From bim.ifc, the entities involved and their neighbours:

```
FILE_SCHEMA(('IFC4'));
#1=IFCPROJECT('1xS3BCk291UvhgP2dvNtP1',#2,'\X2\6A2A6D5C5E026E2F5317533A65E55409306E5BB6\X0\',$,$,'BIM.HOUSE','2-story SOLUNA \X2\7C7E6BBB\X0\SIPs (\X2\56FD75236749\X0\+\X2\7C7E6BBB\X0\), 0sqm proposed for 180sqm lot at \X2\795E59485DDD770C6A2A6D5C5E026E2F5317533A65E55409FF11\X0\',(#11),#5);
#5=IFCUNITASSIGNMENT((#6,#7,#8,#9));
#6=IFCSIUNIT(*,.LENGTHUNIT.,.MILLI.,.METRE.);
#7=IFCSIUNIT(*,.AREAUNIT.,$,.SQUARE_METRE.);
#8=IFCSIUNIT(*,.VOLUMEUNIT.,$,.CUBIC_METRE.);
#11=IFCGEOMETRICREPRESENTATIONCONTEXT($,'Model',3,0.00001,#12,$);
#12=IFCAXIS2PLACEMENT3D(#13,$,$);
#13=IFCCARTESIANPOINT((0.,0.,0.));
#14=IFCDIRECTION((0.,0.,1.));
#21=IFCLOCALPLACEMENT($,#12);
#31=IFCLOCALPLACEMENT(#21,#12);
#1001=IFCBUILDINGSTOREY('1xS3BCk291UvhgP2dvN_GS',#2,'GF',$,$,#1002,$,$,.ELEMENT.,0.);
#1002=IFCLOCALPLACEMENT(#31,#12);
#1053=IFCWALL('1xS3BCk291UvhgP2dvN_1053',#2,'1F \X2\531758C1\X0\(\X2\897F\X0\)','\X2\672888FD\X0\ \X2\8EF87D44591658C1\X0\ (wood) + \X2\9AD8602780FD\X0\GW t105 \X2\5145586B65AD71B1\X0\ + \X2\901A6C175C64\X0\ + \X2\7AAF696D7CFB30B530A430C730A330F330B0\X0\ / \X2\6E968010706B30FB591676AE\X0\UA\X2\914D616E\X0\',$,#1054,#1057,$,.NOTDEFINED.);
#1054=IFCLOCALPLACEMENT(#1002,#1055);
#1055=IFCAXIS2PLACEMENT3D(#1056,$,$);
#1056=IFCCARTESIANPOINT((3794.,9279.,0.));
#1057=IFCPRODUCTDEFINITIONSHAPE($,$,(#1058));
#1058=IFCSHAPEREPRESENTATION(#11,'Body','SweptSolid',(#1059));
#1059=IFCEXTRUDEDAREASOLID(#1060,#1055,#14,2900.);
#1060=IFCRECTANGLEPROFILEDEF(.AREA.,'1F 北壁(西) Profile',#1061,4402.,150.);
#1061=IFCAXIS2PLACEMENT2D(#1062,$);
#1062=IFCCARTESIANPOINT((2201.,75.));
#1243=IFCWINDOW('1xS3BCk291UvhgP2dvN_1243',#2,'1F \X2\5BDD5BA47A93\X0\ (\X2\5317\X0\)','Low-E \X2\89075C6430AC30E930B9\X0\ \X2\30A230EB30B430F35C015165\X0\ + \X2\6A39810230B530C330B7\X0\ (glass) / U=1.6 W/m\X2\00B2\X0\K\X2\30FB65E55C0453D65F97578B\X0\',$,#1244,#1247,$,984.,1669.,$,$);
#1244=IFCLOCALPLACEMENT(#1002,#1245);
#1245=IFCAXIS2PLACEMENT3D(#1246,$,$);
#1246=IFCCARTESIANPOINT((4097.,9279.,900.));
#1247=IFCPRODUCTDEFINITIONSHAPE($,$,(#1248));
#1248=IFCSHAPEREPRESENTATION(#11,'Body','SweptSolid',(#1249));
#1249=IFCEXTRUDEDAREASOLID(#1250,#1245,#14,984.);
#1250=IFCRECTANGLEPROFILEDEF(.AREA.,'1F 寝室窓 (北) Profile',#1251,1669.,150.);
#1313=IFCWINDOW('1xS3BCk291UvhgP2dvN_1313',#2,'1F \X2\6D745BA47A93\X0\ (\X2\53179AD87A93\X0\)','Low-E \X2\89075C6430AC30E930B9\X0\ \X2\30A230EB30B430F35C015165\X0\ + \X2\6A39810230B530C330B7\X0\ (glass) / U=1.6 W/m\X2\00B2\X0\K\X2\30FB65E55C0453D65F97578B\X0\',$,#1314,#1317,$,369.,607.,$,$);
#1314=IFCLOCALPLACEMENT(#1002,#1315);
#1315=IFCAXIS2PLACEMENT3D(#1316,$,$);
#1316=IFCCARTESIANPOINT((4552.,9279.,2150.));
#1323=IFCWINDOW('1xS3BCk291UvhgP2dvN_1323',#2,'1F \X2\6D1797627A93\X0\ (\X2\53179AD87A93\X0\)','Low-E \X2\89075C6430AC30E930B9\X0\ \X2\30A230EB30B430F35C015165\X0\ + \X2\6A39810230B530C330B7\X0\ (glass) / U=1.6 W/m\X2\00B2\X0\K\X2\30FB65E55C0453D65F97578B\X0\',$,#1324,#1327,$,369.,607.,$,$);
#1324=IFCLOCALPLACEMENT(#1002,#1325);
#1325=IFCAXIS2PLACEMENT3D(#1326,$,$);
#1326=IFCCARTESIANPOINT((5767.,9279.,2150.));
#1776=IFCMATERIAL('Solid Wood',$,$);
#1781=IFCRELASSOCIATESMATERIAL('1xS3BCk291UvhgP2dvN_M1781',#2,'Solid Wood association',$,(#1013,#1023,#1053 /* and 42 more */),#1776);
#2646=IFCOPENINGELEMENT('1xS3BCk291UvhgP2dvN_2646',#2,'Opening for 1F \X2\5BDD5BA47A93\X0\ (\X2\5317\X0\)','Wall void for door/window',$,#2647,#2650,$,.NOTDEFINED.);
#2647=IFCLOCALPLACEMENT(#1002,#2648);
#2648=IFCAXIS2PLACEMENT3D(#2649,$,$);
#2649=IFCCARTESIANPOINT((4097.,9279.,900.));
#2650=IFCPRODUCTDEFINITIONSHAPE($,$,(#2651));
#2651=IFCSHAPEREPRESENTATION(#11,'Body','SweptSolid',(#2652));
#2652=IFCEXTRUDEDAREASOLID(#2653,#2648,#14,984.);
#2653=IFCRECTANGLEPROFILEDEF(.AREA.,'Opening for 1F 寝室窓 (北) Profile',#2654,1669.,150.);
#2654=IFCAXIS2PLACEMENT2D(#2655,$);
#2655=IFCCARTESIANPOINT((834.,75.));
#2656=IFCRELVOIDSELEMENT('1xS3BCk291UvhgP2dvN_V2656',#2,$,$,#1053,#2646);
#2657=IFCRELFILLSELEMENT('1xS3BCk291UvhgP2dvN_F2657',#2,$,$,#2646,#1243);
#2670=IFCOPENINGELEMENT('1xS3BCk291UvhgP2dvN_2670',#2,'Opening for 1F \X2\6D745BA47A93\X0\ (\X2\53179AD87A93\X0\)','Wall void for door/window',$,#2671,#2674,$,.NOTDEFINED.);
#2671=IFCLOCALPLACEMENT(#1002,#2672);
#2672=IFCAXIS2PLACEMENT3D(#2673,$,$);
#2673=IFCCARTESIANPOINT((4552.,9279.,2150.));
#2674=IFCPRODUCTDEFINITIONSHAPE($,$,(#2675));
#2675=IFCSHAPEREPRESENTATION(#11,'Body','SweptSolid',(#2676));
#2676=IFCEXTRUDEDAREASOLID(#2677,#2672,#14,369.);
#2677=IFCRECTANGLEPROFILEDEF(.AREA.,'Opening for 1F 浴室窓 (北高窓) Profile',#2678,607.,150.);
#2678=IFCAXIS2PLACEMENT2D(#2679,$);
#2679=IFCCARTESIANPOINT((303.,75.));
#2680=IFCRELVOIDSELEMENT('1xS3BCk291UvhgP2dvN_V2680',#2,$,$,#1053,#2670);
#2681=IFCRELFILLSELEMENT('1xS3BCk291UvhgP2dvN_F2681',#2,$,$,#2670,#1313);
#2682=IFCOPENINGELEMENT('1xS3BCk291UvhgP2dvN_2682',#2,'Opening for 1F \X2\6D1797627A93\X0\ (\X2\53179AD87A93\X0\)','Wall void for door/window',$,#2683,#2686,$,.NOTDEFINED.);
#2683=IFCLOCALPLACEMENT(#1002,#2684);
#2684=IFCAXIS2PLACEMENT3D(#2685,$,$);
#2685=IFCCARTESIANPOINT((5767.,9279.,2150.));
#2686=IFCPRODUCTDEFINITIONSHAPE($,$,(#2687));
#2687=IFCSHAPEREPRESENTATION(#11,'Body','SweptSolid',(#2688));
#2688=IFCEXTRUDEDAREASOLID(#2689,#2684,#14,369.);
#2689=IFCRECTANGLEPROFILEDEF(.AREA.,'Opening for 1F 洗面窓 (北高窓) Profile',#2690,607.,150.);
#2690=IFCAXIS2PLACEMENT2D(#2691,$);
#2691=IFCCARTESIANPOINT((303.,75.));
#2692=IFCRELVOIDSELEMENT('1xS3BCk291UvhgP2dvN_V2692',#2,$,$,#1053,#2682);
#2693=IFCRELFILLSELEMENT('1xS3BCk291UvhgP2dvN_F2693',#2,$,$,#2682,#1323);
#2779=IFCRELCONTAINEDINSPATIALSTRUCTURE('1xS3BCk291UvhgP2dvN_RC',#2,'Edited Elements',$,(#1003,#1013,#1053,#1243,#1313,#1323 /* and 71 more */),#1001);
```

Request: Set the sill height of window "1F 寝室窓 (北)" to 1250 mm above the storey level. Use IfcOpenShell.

```python
import numpy as np
import ifcopenshell
import ifcopenshell.api.geometry
import ifcopenshell.geom
import ifcopenshell.util.element
import ifcopenshell.util.placement
import ifcopenshell.util.shape
import ifcopenshell.util.unit

model = ifcopenshell.open("bim.ifc")
unit_scale = ifcopenshell.util.unit.calculate_unit_scale(model)

window = model.by_guid("1xS3BCk291UvhgP2dvN_1243")
opening = window.FillsVoids[0].RelatingOpeningElement
storey = ifcopenshell.util.element.get_container(window, ifc_class="IfcBuildingStorey")
level = ifcopenshell.util.placement.get_local_placement(storey.ObjectPlacement)[2, 3]

# The opening's origin need not be at the sill, so measure its lowest point.
shape = ifcopenshell.geom.create_shape(ifcopenshell.geom.settings(), opening)
bottom = ifcopenshell.util.shape.get_shape_bottom_elevation(shape, shape.geometry) / unit_scale
dz = level + 1250.0 - bottom

shift = np.array([0.0, 0.0, dz])
# The window is not placed relative to its opening, so move both.
for product in (opening, window):
    matrix = ifcopenshell.util.placement.get_local_placement(product.ObjectPlacement)
    matrix[:3, 3] += shift
    ifcopenshell.api.geometry.edit_object_placement(model, product=product, matrix=matrix, is_si=False)

print(f"moved by {dz * unit_scale:+.3f} m")

model.write("bim_updated.ifc")
```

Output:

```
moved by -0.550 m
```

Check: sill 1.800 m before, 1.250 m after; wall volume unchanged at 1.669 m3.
